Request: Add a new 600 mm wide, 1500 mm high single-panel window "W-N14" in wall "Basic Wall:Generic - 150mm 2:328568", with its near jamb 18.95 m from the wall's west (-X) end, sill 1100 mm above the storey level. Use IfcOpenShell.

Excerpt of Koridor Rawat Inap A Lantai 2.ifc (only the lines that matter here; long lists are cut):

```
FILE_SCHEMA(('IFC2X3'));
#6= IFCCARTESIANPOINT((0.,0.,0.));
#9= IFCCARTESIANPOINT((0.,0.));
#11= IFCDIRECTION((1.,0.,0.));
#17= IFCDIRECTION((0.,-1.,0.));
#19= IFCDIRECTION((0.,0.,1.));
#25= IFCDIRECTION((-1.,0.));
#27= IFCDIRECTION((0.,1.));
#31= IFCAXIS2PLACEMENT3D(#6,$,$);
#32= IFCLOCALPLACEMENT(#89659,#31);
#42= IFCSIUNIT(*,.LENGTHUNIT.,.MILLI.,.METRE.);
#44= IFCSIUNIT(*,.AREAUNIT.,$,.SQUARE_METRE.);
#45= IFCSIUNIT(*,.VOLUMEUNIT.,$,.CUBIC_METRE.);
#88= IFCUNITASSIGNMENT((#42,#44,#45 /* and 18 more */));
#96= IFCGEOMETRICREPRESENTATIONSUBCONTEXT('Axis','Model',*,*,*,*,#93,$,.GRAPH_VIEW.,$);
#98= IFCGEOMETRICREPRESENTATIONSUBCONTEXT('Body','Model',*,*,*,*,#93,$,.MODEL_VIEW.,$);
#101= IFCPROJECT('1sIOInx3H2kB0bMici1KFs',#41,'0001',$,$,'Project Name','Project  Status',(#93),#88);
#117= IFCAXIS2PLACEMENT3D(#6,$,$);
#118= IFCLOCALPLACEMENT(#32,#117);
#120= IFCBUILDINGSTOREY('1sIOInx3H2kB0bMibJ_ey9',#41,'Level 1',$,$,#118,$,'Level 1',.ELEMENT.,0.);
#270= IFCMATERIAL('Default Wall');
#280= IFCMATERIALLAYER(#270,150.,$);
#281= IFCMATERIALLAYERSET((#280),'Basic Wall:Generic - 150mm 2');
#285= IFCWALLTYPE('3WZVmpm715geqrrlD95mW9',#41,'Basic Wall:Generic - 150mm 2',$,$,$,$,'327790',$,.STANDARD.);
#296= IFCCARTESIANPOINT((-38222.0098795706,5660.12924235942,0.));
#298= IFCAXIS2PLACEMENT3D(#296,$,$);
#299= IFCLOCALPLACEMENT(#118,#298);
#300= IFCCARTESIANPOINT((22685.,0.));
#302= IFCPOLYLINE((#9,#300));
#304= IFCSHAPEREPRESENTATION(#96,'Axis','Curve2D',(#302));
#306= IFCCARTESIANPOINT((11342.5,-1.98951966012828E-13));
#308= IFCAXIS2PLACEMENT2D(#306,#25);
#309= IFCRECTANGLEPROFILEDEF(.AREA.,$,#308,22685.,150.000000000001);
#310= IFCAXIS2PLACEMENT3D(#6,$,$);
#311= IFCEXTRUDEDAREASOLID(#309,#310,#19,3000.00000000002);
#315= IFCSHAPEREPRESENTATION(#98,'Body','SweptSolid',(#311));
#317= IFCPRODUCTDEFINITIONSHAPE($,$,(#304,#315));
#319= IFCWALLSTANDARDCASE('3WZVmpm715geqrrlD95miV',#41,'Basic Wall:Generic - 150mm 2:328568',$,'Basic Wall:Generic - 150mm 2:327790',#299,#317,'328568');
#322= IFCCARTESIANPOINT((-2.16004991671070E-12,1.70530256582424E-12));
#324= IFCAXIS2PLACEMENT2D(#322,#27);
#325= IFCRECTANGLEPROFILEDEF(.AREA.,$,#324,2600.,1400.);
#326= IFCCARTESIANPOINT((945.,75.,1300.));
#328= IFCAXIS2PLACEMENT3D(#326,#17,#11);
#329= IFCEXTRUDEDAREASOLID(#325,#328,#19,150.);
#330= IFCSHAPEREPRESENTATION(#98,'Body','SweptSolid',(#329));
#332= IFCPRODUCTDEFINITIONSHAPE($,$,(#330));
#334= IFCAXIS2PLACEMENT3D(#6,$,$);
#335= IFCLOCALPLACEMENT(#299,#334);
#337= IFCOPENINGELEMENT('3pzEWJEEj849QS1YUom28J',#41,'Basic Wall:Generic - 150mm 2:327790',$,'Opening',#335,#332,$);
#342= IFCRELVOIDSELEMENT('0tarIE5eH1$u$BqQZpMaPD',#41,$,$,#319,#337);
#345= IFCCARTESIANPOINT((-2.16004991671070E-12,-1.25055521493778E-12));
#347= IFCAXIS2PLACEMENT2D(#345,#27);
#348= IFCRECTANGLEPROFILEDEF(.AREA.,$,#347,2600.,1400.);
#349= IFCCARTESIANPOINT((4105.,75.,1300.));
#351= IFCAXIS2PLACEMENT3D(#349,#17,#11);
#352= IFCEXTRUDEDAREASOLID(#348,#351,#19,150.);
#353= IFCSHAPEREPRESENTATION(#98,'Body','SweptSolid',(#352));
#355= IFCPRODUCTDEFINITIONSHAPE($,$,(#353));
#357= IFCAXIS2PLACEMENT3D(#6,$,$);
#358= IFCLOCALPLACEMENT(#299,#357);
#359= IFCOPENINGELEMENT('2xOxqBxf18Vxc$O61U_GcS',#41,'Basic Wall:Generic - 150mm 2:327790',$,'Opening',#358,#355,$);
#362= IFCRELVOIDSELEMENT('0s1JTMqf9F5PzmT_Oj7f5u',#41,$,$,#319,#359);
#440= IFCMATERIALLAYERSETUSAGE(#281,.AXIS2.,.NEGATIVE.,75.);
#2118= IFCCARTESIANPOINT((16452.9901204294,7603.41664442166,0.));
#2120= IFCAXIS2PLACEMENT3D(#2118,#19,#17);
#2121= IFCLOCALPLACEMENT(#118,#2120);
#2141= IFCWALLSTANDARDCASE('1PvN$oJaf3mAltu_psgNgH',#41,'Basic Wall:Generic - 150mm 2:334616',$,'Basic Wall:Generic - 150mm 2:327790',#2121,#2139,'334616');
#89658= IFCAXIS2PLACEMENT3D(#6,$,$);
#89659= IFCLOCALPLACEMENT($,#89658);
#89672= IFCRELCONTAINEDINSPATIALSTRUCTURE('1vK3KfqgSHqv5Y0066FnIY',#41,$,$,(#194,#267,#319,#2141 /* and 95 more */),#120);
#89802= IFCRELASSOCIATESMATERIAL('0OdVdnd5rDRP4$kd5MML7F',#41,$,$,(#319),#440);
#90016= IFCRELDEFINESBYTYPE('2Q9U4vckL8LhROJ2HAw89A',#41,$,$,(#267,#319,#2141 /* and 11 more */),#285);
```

```python
import numpy as np
import ifcopenshell
import ifcopenshell.api.feature
import ifcopenshell.api.geometry
import ifcopenshell.api.root
import ifcopenshell.api.spatial
import ifcopenshell.api.type
import ifcopenshell.geom
import ifcopenshell.util.element
import ifcopenshell.util.placement
import ifcopenshell.util.representation
import ifcopenshell.util.shape
import ifcopenshell.util.unit

model = ifcopenshell.open("Koridor Rawat Inap A Lantai 2.ifc")
unit_scale = ifcopenshell.util.unit.calculate_unit_scale(model)
settings = ifcopenshell.geom.settings()


def volume(element):
    """Net volume in cubic metres, openings subtracted."""
    shape = ifcopenshell.geom.create_shape(settings, element)
    return ifcopenshell.util.shape.get_volume(shape.geometry)


wall = model.by_guid("3WZVmpm715geqrrlD95miV")
storey = ifcopenshell.util.element.get_container(wall, ifc_class="IfcBuildingStorey")
context = ifcopenshell.util.representation.get_context(model, "Model", "Body", "MODEL_VIEW")
before = volume(wall)

width, height, from_end, sill = 0.6, 1.5, 18.95, 1.1  # metres

# The wall runs along its own X axis, and the end named is its -X end.
wall_shape = ifcopenshell.geom.create_shape(settings, wall)
x, y, z = ifcopenshell.util.shape.get_vertices(wall_shape.geometry).T
start = x.min() + from_end
face, thickness = float(y.min()), float(y.max() - y.min())
wall_matrix = ifcopenshell.util.placement.get_local_placement(wall.ObjectPlacement)
level = ifcopenshell.util.placement.get_local_placement(storey.ObjectPlacement)[2, 3]


def in_wall(x, y):
    """Placement at x, y metres in the wall's axes, at sill height."""
    matrix = wall_matrix.copy()
    matrix[:, 3] = wall_matrix @ np.array([x / unit_scale, y / unit_scale, 0.0, 1.0])
    matrix[2, 3] = level + sill / unit_scale
    return matrix


# Opening: a box that overshoots both wall faces by 50 mm.
opening = ifcopenshell.api.root.create_entity(model, ifc_class="IfcOpeningElement")
box = ifcopenshell.api.geometry.add_wall_representation(
    model, context=context, length=width, height=height, thickness=thickness + 0.1
)
ifcopenshell.api.geometry.assign_representation(model, product=opening, representation=box)
ifcopenshell.api.geometry.edit_object_placement(model, product=opening, matrix=in_wall(start, face - 0.05), is_si=False)
ifcopenshell.api.feature.add_feature(model, feature=opening, element=wall)

window = ifcopenshell.api.root.create_entity(model, ifc_class="IfcWindow", name="W-N14")
window.OverallWidth, window.OverallHeight = width / unit_scale, height / unit_scale
body = ifcopenshell.api.geometry.add_window_representation(
    model,
    context=context,
    overall_width=window.OverallWidth,
    overall_height=window.OverallHeight,
    partition_type="SINGLE_PANEL",
)
ifcopenshell.api.geometry.assign_representation(model, product=window, representation=body)
ifcopenshell.api.spatial.assign_container(model, products=[window], relating_structure=storey)
fills = ifcopenshell.api.feature.add_filling(model, opening=opening, element=window)
fills.OwnerHistory = window.OwnerHistory  # required in IFC2X3

# IFC2X3 keeps the operation on the window style.
style = ifcopenshell.api.root.create_entity(model, ifc_class="IfcWindowStyle", name="W-N14")
style.OperationType, style.ConstructionType = "SINGLE_PANEL", "NOTDEFINED"
style.ParameterTakesPrecedence = style.Sizeable = False
ifcopenshell.api.type.assign_type(model, related_objects=[window], relating_type=style)

# Centre the window in the wall's thickness.
ifcopenshell.api.geometry.edit_object_placement(model, product=window, matrix=in_wall(start, face), is_si=False)
window_shape = ifcopenshell.geom.create_shape(settings, window)
depth = ifcopenshell.util.shape.get_vertices(window_shape.geometry)[:, 1]
offset = face + thickness / 2 - (depth.min() + depth.max()) / 2
ifcopenshell.api.geometry.edit_object_placement(model, product=window, matrix=in_wall(start, offset), is_si=False)

after = volume(wall)

print(f"wall volume {before:.3f} -> {after:.3f} m3")

model.write("Koridor Rawat Inap A Lantai 2_updated.ifc")
```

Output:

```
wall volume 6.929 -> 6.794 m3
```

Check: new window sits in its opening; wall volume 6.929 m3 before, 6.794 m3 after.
